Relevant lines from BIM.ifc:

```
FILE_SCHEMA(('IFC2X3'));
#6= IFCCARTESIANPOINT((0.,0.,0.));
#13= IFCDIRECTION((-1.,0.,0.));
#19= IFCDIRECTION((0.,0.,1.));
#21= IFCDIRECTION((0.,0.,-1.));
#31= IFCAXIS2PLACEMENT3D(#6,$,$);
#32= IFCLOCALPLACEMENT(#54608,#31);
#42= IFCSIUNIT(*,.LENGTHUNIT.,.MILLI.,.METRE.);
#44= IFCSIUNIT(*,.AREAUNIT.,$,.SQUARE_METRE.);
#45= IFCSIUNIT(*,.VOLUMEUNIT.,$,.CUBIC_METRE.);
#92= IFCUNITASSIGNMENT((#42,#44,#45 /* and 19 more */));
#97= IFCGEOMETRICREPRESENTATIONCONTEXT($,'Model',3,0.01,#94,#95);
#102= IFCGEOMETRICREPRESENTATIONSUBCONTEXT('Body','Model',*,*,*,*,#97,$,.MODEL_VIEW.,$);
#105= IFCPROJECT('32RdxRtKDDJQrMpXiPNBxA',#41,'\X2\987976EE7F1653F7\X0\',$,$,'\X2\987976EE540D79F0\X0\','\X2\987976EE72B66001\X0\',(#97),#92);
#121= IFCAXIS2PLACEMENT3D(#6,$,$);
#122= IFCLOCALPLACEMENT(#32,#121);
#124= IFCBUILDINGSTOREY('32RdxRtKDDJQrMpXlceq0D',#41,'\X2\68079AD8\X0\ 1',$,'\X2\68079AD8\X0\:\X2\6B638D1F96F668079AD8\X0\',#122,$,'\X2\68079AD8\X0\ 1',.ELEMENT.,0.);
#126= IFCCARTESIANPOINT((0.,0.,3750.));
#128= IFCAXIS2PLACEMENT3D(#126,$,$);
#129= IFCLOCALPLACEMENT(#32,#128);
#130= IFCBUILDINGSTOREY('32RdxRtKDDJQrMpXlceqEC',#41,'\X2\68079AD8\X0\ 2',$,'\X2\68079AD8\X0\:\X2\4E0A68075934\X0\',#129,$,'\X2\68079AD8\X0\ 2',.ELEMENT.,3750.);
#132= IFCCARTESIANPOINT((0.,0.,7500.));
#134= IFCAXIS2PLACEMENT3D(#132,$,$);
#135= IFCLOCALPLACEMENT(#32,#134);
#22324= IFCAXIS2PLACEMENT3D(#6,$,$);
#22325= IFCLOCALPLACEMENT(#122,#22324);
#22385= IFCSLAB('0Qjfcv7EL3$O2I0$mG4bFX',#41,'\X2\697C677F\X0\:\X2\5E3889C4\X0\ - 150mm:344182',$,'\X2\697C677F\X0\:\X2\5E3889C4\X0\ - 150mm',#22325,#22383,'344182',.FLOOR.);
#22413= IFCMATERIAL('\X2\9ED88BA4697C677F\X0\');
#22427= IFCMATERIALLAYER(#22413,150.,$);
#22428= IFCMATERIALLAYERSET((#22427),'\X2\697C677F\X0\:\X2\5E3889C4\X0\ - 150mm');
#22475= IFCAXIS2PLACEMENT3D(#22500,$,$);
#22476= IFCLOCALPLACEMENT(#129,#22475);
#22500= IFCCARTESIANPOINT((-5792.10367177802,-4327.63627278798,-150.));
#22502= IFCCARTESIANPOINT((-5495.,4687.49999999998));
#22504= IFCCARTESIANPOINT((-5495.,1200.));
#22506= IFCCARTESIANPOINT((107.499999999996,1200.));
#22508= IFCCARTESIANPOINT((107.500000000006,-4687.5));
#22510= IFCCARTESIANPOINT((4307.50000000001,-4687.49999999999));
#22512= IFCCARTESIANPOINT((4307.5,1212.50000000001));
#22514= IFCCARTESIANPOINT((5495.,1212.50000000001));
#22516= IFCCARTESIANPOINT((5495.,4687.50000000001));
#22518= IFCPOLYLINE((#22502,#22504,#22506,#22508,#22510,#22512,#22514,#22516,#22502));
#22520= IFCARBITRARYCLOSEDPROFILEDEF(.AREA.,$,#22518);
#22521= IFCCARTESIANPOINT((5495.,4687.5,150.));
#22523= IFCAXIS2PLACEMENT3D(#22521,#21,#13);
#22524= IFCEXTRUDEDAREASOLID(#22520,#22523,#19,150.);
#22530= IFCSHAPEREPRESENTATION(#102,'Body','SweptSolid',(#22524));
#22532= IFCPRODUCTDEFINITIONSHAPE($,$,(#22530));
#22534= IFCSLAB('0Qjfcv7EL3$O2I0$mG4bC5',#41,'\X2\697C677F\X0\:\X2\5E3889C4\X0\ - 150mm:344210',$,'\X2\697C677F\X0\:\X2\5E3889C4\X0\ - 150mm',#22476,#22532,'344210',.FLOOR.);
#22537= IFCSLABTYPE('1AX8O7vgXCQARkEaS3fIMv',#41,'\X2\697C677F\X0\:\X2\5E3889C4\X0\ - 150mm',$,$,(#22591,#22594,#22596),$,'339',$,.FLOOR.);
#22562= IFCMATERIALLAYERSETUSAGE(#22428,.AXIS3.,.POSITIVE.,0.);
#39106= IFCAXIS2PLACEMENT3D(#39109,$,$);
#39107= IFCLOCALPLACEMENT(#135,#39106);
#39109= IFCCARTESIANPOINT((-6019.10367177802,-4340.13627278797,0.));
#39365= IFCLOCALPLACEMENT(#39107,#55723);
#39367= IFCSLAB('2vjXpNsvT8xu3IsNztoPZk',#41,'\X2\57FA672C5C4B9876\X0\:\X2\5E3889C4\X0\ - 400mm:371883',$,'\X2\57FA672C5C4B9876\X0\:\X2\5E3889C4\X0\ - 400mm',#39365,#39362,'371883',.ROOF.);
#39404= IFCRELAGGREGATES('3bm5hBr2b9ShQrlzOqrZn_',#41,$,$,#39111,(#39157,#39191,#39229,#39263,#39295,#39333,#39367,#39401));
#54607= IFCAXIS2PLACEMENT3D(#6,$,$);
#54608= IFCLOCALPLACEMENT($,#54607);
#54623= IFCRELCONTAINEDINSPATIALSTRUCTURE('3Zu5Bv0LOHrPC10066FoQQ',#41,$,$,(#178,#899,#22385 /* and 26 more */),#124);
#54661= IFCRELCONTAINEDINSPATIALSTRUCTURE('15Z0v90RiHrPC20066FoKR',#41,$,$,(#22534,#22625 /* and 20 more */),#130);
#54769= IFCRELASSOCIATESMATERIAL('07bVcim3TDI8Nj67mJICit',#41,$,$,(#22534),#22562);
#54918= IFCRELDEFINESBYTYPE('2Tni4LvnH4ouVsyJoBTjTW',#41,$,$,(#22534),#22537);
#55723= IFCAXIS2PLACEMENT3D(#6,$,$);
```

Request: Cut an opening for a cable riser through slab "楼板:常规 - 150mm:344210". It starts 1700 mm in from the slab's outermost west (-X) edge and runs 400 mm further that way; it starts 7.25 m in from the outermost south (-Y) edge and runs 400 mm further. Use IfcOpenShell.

```python
import numpy as np
import ifcopenshell
import ifcopenshell.api.feature
import ifcopenshell.api.geometry
import ifcopenshell.api.root
import ifcopenshell.geom
import ifcopenshell.util.placement
import ifcopenshell.util.representation
import ifcopenshell.util.shape
import ifcopenshell.util.unit

model = ifcopenshell.open("BIM.ifc")
unit_scale = ifcopenshell.util.unit.calculate_unit_scale(model)
settings = ifcopenshell.geom.settings()


def volume(element):
    """Net volume in cubic metres, openings subtracted."""
    shape = ifcopenshell.geom.create_shape(settings, element)
    return ifcopenshell.util.shape.get_volume(shape.geometry)


slab = model.by_guid("0Qjfcv7EL3$O2I0$mG4bC5")
before = volume(slab)

# Extent in the slab's own axes, in metres. The edges named are its -X and -Y sides.
slab_shape = ifcopenshell.geom.create_shape(settings, slab)
vertices = ifcopenshell.util.shape.get_vertices(slab_shape.geometry)
x_min, y_min, bottom = vertices.min(axis=0)
top = vertices[:, 2].max()

opening = ifcopenshell.api.root.create_entity(model, ifc_class="IfcOpeningElement", name="Cable riser opening")
context = ifcopenshell.util.representation.get_context(model, "Model", "Body", "MODEL_VIEW")
width, depth = 0.4, 0.4
outline = [(0.0, 0.0), (width, 0.0), (width, depth), (0.0, depth), (0.0, 0.0)]
# Overshoot both faces by 50 mm so the cut is clean.
shape = ifcopenshell.api.geometry.add_slab_representation(
    model, context=context, depth=top - bottom + 0.1, polyline=outline
)
ifcopenshell.api.geometry.assign_representation(model, product=opening, representation=shape)

matrix = ifcopenshell.util.placement.get_local_placement(slab.ObjectPlacement)
matrix[:, 3] = matrix @ np.append(np.array([x_min + 1.7, y_min + 7.25, bottom - 0.05]) / unit_scale, 1.0)
ifcopenshell.api.geometry.edit_object_placement(model, product=opening, matrix=matrix, is_si=False)
ifcopenshell.api.feature.add_feature(model, feature=opening, element=slab)

after = volume(slab)

print(f"slab volume {before:.3f} -> {after:.3f} m3")

model.write("BIM_updated.ifc")
```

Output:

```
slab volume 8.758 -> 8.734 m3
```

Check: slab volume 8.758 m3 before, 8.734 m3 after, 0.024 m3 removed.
